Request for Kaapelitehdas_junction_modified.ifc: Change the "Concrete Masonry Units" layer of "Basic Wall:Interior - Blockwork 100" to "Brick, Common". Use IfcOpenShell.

First a look at what the model holds.

```python
import ifcopenshell
import ifcopenshell.util.element

model = ifcopenshell.open("Kaapelitehdas_junction_modified.ifc")
print(model.schema)
for layer_set in model.by_type("IfcMaterialLayerSet"):
    if layer_set.LayerSetName == "Basic Wall:Interior - Blockwork 100":
        for layer in layer_set.MaterialLayers:
            print(layer.id(), layer.Material and layer.Material.Name, layer.LayerThickness, sep=" | ")
        print(len(ifcopenshell.util.element.get_elements_by_material(model, layer_set)), "elements and types use it")
print(sorted(m.Name for m in model.by_type("IfcMaterial") if m.Name)[:60])
```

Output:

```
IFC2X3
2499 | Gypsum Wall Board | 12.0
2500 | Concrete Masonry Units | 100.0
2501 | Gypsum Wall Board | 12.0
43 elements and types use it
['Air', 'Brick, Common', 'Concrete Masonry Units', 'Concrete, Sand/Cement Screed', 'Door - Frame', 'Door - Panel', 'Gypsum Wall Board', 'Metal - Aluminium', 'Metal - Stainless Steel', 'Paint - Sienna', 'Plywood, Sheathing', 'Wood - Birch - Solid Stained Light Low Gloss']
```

```python
import ifcopenshell
import ifcopenshell.api.material

model = ifcopenshell.open("Kaapelitehdas_junction_modified.ifc")

layer_set = next(s for s in model.by_type("IfcMaterialLayerSet") if s.LayerSetName == "Basic Wall:Interior - Blockwork 100")
layer = next(l for l in layer_set.MaterialLayers if l.Material and l.Material.Name == "Concrete Masonry Units")
material = next(m for m in model.by_type("IfcMaterial") if m.Name == "Brick, Common")

# Point this one layer at the other material; renaming the old one would change it everywhere.
ifcopenshell.api.material.edit_layer(model, layer=layer, attributes={}, material=material)

print([l.Material.Name if l.Material else None for l in layer_set.MaterialLayers])

model.write("Kaapelitehdas_junction_modified_edited.ifc")
```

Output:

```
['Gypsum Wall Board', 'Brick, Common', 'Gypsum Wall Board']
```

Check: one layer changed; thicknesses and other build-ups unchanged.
